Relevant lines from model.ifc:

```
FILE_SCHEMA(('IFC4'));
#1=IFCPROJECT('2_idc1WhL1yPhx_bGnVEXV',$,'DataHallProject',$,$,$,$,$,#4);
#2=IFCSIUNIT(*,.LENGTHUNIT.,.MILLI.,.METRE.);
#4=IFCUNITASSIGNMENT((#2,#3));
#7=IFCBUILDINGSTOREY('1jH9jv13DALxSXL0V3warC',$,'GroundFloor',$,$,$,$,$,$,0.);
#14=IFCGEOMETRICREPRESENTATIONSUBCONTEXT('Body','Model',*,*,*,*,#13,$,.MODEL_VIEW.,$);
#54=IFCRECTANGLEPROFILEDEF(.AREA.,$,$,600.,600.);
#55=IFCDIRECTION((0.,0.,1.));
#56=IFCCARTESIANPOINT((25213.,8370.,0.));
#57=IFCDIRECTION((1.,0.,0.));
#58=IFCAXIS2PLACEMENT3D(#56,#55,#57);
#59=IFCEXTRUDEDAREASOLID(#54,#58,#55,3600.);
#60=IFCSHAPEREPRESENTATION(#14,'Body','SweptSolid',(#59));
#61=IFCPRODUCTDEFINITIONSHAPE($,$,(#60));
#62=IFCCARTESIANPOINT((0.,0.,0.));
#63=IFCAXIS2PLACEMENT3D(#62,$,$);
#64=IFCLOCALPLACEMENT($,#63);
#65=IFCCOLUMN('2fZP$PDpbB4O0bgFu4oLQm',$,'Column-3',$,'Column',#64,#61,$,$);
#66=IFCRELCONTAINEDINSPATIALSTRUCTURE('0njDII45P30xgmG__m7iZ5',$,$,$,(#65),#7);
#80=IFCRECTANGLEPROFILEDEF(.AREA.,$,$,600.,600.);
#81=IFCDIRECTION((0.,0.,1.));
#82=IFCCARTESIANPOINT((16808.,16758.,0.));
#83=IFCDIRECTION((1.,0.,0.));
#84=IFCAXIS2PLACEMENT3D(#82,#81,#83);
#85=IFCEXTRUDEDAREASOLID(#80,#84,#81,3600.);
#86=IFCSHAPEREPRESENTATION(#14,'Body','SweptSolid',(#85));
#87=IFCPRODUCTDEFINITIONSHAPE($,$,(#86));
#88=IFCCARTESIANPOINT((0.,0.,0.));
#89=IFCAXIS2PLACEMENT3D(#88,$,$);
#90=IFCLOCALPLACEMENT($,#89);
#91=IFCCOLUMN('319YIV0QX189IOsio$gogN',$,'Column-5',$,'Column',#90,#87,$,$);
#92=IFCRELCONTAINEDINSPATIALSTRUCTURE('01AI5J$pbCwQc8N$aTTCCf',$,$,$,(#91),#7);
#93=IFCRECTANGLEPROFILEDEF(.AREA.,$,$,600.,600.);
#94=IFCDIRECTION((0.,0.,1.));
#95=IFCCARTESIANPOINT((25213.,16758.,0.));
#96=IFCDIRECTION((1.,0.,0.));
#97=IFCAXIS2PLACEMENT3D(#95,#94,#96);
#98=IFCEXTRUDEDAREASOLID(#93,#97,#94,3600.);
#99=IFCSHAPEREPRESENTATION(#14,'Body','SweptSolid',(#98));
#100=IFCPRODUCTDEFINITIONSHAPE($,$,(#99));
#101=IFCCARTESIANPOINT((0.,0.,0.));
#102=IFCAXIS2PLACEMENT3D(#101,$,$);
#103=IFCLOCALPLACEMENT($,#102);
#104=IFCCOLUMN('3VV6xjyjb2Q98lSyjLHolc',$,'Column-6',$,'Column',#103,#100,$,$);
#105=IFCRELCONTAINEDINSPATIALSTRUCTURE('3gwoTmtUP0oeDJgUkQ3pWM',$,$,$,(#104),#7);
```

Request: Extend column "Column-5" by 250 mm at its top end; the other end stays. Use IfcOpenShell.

```python
import ifcopenshell
import ifcopenshell.util.representation
import ifcopenshell.util.unit

model = ifcopenshell.open("model.ifc")
unit_scale = ifcopenshell.util.unit.calculate_unit_scale(model)

member = model.by_guid("319YIV0QX189IOsio$gogN")
change = 0.25 / unit_scale

# The extrusion runs towards the end named, so only its depth changes.
body = ifcopenshell.util.representation.get_representation(member, "Model", "Body")
solid = body.Items[0]
old_length = solid.Depth
solid.Depth += change

print(f"length {old_length:g} -> {solid.Depth:g}")

model.write("model_edited.ifc")
```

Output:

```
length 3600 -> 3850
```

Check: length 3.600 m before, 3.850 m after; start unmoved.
